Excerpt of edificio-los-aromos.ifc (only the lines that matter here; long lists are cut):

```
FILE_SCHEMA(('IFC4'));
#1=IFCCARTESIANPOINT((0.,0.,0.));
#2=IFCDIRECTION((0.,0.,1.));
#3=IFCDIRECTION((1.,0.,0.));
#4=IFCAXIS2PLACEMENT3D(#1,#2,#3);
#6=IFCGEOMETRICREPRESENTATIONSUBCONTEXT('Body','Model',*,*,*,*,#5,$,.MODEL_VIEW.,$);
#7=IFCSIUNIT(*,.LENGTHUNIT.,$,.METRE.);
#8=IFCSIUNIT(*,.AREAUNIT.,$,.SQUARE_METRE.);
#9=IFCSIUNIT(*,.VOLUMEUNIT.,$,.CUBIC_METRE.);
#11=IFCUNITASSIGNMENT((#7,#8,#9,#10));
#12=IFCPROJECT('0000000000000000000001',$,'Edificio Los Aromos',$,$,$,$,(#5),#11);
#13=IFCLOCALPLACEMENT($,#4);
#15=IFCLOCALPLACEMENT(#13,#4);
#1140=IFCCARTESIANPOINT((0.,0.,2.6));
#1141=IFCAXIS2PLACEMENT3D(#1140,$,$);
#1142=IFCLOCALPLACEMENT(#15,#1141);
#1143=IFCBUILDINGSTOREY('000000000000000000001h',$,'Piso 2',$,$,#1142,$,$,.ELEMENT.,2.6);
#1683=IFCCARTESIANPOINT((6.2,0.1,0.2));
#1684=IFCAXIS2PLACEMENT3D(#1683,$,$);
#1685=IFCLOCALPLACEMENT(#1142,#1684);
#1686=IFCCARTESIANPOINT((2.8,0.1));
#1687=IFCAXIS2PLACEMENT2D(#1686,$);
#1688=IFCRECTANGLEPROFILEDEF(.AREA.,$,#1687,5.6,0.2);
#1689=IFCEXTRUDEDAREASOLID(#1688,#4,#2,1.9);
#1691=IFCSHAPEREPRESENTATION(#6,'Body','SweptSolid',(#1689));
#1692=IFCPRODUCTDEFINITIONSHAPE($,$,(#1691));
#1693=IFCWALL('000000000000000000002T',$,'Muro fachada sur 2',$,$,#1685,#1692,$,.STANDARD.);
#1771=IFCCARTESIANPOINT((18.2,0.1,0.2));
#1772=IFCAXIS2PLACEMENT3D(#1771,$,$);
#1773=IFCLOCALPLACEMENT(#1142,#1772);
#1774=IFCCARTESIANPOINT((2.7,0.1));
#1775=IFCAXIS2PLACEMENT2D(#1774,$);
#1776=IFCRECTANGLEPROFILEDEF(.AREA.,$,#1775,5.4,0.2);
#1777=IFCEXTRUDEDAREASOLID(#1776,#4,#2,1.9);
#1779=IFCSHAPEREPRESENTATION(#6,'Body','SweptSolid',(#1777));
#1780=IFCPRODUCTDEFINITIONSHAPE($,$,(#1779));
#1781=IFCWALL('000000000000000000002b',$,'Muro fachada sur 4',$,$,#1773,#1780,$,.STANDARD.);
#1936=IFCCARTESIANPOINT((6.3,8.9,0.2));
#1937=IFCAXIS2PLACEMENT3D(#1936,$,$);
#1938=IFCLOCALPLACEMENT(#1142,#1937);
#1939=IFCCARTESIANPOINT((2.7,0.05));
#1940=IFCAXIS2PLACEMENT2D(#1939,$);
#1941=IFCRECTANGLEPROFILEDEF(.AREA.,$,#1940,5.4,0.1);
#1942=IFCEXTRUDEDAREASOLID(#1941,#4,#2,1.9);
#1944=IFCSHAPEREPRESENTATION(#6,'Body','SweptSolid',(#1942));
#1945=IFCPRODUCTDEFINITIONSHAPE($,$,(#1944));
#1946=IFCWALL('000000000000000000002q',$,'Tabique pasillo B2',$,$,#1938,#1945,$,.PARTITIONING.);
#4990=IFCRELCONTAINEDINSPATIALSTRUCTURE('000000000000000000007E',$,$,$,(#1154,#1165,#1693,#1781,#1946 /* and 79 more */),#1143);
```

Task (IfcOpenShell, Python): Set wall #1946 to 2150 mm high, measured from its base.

```python
import ifcopenshell
import ifcopenshell.geom
import ifcopenshell.util.representation
import ifcopenshell.util.shape
import ifcopenshell.util.unit

model = ifcopenshell.open("edificio-los-aromos.ifc")
unit_scale = ifcopenshell.util.unit.calculate_unit_scale(model)
settings = ifcopenshell.geom.settings()


def volume(element):
    """Net volume in cubic metres, openings subtracted."""
    shape = ifcopenshell.geom.create_shape(settings, element)
    return ifcopenshell.util.shape.get_volume(shape.geometry)


wall = model.by_id(1946)
before = volume(wall)

body = ifcopenshell.util.representation.get_representation(wall, "Model", "Body")
solid = body.Items[0]
old_height = solid.Depth
solid.Depth = 2.15 / unit_scale
after = volume(wall)

print(f"height {old_height:g} -> {solid.Depth:g}, volume {before:.3f} -> {after:.3f} m3")

model.write("edificio-los-aromos_edited.ifc")
```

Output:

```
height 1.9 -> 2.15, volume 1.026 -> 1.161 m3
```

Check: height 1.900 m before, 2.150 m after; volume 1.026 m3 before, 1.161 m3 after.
